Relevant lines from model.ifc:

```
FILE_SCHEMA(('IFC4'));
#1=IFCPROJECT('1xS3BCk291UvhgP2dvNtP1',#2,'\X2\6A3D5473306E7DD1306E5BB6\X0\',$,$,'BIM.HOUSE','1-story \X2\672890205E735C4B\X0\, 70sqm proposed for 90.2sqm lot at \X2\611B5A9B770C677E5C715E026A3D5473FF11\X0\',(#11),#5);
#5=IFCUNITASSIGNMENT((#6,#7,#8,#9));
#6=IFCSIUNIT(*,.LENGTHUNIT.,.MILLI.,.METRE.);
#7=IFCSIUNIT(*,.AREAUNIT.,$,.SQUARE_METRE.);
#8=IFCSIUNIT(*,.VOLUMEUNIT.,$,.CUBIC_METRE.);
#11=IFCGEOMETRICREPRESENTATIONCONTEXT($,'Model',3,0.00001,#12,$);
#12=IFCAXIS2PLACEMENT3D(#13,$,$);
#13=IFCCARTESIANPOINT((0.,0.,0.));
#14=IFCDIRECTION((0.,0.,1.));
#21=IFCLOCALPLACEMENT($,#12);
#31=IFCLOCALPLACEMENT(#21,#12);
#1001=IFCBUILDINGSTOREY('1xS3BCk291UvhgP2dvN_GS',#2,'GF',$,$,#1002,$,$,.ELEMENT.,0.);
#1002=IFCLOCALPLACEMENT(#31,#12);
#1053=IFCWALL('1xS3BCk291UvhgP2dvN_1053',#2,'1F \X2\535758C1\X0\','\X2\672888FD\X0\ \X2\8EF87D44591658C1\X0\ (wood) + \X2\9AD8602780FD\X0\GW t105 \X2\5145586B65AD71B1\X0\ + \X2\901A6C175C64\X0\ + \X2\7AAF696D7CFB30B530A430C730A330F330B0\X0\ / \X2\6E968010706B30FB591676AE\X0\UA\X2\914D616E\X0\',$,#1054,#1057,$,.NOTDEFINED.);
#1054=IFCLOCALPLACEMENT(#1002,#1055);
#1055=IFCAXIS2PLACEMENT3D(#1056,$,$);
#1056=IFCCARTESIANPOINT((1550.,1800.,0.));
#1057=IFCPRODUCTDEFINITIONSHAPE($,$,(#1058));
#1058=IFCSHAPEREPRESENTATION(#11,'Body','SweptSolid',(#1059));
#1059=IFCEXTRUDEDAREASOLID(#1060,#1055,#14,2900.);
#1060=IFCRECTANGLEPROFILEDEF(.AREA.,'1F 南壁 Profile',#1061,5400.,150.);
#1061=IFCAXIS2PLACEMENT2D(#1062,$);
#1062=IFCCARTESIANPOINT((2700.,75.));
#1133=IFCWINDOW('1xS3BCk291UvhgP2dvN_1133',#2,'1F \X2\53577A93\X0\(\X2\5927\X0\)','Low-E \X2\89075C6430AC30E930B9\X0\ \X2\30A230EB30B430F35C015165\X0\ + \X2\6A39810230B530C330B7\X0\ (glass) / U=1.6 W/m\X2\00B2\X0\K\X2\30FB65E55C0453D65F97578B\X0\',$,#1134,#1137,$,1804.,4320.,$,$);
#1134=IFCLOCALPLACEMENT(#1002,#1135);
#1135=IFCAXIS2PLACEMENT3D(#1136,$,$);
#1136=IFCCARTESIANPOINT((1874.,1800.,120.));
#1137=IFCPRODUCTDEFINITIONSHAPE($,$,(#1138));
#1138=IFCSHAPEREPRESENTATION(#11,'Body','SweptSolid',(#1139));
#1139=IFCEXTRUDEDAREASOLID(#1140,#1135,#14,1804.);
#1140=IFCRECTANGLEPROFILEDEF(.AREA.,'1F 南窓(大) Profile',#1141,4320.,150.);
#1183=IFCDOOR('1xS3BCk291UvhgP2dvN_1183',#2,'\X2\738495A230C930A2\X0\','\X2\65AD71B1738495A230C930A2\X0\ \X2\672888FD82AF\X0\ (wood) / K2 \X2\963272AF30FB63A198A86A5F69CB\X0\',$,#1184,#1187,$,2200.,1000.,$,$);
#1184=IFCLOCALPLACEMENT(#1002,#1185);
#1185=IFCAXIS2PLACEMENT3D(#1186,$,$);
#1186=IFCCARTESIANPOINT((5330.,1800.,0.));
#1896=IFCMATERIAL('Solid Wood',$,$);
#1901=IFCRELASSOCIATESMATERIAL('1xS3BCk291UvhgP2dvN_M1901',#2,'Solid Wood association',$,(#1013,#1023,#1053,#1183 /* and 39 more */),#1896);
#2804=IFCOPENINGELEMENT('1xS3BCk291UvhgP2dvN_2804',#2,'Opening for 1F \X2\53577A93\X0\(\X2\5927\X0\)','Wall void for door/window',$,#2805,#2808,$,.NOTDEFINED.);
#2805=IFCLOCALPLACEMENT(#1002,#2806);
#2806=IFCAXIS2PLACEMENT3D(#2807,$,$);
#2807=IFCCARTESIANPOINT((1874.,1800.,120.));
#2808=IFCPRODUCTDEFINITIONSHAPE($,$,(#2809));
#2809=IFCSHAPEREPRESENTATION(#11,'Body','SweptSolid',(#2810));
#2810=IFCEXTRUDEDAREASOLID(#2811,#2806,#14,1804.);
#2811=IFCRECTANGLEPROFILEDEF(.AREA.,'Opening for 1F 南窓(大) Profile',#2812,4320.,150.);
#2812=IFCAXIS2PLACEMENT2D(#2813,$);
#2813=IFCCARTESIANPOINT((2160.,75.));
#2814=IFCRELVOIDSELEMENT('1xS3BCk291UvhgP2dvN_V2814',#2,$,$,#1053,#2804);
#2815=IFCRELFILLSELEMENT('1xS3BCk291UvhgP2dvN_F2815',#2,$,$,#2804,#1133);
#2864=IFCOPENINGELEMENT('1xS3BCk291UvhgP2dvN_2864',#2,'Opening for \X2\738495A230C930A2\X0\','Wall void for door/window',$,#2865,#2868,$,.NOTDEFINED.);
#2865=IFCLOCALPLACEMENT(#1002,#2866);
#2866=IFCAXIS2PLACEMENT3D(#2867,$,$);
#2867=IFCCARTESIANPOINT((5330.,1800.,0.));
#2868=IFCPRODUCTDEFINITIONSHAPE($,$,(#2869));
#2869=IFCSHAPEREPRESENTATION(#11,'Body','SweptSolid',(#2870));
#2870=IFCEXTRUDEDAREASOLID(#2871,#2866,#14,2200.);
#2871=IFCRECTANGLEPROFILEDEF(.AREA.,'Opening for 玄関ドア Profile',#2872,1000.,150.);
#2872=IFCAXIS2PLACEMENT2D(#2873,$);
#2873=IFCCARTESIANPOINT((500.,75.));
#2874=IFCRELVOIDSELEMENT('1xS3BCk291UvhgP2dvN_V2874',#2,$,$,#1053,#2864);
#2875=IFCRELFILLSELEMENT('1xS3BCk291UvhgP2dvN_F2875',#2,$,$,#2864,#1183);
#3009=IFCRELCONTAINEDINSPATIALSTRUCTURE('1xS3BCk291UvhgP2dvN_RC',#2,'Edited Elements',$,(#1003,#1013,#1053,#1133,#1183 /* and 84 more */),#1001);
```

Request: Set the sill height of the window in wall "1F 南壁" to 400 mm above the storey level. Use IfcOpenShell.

```python
import numpy as np
import ifcopenshell
import ifcopenshell.api.geometry
import ifcopenshell.geom
import ifcopenshell.util.element
import ifcopenshell.util.placement
import ifcopenshell.util.shape
import ifcopenshell.util.unit

model = ifcopenshell.open("model.ifc")
unit_scale = ifcopenshell.util.unit.calculate_unit_scale(model)

window = model.by_guid("1xS3BCk291UvhgP2dvN_1133")
opening = window.FillsVoids[0].RelatingOpeningElement
storey = ifcopenshell.util.element.get_container(window, ifc_class="IfcBuildingStorey")
level = ifcopenshell.util.placement.get_local_placement(storey.ObjectPlacement)[2, 3]

# The opening's origin need not be at the sill, so measure its lowest point.
shape = ifcopenshell.geom.create_shape(ifcopenshell.geom.settings(), opening)
bottom = ifcopenshell.util.shape.get_shape_bottom_elevation(shape, shape.geometry) / unit_scale
dz = level + 400.0 - bottom

shift = np.array([0.0, 0.0, dz])
# The window is not placed relative to its opening, so move both.
for product in (opening, window):
    matrix = ifcopenshell.util.placement.get_local_placement(product.ObjectPlacement)
    matrix[:3, 3] += shift
    ifcopenshell.api.geometry.edit_object_placement(model, product=product, matrix=matrix, is_si=False)

print(f"moved by {dz * unit_scale:+.3f} m")

model.write("model_edited.ifc")
```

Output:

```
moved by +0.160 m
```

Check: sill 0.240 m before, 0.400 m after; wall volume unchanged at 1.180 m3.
